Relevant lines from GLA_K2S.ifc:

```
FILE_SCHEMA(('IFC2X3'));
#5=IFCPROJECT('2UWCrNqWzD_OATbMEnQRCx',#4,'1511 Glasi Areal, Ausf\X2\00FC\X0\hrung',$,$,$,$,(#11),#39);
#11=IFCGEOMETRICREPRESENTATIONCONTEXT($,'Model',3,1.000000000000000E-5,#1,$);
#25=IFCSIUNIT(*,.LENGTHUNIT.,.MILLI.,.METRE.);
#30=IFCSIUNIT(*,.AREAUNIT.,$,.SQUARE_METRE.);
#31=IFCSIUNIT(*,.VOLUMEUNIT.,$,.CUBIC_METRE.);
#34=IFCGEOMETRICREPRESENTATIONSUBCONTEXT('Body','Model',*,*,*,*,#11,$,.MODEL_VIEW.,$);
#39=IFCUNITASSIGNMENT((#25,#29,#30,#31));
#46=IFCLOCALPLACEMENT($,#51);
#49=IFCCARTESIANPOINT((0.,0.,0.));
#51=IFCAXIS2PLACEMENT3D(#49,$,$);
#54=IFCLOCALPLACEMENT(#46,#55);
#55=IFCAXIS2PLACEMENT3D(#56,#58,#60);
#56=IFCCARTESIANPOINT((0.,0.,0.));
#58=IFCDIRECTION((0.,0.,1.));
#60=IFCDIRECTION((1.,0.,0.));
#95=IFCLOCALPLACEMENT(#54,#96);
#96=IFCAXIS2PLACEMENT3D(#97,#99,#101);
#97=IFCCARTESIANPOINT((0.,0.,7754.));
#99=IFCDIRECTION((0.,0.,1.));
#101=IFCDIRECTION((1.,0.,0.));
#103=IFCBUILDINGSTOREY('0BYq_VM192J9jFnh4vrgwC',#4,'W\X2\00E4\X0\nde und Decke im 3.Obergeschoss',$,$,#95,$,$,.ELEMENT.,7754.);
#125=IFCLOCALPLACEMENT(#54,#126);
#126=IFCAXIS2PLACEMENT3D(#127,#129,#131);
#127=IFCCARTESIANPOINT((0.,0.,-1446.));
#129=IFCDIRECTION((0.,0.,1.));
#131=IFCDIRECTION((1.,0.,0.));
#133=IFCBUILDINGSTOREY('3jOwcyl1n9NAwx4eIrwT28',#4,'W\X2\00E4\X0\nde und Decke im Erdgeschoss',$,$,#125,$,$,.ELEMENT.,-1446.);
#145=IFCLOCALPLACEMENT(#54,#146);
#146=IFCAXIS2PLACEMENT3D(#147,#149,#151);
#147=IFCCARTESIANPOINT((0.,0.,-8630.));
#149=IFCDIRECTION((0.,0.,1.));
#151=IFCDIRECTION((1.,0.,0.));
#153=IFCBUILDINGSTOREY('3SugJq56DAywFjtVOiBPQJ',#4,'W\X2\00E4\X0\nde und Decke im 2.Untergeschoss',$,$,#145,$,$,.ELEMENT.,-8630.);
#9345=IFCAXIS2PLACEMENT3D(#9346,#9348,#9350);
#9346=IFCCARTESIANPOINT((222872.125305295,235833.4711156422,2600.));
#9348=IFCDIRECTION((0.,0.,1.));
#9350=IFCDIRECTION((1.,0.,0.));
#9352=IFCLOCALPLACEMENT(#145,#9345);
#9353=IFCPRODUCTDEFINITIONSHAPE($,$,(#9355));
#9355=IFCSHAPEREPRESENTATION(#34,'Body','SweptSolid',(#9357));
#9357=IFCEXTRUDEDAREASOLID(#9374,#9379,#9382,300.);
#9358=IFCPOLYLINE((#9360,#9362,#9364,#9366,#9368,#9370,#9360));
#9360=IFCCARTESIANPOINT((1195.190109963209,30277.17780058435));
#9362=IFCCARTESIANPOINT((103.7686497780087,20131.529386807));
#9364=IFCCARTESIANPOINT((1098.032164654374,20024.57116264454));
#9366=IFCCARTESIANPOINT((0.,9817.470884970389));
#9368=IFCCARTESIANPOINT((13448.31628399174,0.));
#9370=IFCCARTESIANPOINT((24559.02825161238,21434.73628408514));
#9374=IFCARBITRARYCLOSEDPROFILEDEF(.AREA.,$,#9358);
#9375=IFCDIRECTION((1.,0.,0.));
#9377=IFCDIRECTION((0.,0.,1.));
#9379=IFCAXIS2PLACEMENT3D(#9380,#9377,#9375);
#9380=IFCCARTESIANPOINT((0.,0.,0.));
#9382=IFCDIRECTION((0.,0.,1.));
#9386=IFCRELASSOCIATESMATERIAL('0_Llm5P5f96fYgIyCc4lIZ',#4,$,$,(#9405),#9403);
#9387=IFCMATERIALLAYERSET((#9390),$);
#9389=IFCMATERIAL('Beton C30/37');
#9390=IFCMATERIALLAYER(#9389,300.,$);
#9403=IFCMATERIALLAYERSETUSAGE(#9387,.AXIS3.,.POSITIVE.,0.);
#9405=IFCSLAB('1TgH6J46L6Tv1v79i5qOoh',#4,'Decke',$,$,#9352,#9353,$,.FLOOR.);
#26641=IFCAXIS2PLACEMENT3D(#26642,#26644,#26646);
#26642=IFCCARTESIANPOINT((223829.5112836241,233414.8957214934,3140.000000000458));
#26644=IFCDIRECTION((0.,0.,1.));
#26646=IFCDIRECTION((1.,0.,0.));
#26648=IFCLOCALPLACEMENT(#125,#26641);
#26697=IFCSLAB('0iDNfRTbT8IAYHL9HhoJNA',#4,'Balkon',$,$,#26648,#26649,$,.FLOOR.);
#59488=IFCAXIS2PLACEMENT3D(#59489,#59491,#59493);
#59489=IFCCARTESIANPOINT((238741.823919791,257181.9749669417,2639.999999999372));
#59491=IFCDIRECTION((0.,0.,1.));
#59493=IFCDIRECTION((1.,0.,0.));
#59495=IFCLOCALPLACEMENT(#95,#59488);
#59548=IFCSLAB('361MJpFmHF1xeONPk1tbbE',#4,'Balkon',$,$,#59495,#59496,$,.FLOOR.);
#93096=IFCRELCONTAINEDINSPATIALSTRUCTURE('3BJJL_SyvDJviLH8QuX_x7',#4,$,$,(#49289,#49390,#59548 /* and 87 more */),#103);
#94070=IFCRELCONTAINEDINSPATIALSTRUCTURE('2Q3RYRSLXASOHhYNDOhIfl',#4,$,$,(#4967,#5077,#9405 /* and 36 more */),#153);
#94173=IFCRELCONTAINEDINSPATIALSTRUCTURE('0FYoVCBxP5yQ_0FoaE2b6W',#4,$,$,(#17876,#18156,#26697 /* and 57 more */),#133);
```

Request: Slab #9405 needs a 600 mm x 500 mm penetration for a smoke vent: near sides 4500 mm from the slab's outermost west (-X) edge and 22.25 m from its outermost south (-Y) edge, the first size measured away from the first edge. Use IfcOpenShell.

```python
import numpy as np
import ifcopenshell
import ifcopenshell.api.feature
import ifcopenshell.api.geometry
import ifcopenshell.api.root
import ifcopenshell.geom
import ifcopenshell.util.placement
import ifcopenshell.util.representation
import ifcopenshell.util.shape
import ifcopenshell.util.unit

model = ifcopenshell.open("GLA_K2S.ifc")
unit_scale = ifcopenshell.util.unit.calculate_unit_scale(model)
settings = ifcopenshell.geom.settings()


def volume(element):
    """Net volume in cubic metres, openings subtracted."""
    shape = ifcopenshell.geom.create_shape(settings, element)
    return ifcopenshell.util.shape.get_volume(shape.geometry)


slab = model.by_id(9405)
before = volume(slab)

# Extent in the slab's own axes, in metres. The edges named are its -X and -Y sides.
slab_shape = ifcopenshell.geom.create_shape(settings, slab)
vertices = ifcopenshell.util.shape.get_vertices(slab_shape.geometry)
x_min, y_min, bottom = vertices.min(axis=0)
top = vertices[:, 2].max()

opening = ifcopenshell.api.root.create_entity(model, ifc_class="IfcOpeningElement", name="Smoke vent opening")
context = ifcopenshell.util.representation.get_context(model, "Model", "Body", "MODEL_VIEW")
width, depth = 0.6, 0.5
outline = [(0.0, 0.0), (width, 0.0), (width, depth), (0.0, depth), (0.0, 0.0)]
# Overshoot both faces by 50 mm so the cut is clean.
shape = ifcopenshell.api.geometry.add_slab_representation(
    model, context=context, depth=top - bottom + 0.1, polyline=outline
)
ifcopenshell.api.geometry.assign_representation(model, product=opening, representation=shape)

matrix = ifcopenshell.util.placement.get_local_placement(slab.ObjectPlacement)
matrix[:, 3] = matrix @ np.append(np.array([x_min + 4.5, y_min + 22.25, bottom - 0.05]) / unit_scale, 1.0)
ifcopenshell.api.geometry.edit_object_placement(model, product=opening, matrix=matrix, is_si=False)
ifcopenshell.api.feature.add_feature(model, feature=opening, element=slab)

after = volume(slab)

print(f"slab volume {before:.3f} -> {after:.3f} m3")

model.write("GLA_K2S-out.ifc")
```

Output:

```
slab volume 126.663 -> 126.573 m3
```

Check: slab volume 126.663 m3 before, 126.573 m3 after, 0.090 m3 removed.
